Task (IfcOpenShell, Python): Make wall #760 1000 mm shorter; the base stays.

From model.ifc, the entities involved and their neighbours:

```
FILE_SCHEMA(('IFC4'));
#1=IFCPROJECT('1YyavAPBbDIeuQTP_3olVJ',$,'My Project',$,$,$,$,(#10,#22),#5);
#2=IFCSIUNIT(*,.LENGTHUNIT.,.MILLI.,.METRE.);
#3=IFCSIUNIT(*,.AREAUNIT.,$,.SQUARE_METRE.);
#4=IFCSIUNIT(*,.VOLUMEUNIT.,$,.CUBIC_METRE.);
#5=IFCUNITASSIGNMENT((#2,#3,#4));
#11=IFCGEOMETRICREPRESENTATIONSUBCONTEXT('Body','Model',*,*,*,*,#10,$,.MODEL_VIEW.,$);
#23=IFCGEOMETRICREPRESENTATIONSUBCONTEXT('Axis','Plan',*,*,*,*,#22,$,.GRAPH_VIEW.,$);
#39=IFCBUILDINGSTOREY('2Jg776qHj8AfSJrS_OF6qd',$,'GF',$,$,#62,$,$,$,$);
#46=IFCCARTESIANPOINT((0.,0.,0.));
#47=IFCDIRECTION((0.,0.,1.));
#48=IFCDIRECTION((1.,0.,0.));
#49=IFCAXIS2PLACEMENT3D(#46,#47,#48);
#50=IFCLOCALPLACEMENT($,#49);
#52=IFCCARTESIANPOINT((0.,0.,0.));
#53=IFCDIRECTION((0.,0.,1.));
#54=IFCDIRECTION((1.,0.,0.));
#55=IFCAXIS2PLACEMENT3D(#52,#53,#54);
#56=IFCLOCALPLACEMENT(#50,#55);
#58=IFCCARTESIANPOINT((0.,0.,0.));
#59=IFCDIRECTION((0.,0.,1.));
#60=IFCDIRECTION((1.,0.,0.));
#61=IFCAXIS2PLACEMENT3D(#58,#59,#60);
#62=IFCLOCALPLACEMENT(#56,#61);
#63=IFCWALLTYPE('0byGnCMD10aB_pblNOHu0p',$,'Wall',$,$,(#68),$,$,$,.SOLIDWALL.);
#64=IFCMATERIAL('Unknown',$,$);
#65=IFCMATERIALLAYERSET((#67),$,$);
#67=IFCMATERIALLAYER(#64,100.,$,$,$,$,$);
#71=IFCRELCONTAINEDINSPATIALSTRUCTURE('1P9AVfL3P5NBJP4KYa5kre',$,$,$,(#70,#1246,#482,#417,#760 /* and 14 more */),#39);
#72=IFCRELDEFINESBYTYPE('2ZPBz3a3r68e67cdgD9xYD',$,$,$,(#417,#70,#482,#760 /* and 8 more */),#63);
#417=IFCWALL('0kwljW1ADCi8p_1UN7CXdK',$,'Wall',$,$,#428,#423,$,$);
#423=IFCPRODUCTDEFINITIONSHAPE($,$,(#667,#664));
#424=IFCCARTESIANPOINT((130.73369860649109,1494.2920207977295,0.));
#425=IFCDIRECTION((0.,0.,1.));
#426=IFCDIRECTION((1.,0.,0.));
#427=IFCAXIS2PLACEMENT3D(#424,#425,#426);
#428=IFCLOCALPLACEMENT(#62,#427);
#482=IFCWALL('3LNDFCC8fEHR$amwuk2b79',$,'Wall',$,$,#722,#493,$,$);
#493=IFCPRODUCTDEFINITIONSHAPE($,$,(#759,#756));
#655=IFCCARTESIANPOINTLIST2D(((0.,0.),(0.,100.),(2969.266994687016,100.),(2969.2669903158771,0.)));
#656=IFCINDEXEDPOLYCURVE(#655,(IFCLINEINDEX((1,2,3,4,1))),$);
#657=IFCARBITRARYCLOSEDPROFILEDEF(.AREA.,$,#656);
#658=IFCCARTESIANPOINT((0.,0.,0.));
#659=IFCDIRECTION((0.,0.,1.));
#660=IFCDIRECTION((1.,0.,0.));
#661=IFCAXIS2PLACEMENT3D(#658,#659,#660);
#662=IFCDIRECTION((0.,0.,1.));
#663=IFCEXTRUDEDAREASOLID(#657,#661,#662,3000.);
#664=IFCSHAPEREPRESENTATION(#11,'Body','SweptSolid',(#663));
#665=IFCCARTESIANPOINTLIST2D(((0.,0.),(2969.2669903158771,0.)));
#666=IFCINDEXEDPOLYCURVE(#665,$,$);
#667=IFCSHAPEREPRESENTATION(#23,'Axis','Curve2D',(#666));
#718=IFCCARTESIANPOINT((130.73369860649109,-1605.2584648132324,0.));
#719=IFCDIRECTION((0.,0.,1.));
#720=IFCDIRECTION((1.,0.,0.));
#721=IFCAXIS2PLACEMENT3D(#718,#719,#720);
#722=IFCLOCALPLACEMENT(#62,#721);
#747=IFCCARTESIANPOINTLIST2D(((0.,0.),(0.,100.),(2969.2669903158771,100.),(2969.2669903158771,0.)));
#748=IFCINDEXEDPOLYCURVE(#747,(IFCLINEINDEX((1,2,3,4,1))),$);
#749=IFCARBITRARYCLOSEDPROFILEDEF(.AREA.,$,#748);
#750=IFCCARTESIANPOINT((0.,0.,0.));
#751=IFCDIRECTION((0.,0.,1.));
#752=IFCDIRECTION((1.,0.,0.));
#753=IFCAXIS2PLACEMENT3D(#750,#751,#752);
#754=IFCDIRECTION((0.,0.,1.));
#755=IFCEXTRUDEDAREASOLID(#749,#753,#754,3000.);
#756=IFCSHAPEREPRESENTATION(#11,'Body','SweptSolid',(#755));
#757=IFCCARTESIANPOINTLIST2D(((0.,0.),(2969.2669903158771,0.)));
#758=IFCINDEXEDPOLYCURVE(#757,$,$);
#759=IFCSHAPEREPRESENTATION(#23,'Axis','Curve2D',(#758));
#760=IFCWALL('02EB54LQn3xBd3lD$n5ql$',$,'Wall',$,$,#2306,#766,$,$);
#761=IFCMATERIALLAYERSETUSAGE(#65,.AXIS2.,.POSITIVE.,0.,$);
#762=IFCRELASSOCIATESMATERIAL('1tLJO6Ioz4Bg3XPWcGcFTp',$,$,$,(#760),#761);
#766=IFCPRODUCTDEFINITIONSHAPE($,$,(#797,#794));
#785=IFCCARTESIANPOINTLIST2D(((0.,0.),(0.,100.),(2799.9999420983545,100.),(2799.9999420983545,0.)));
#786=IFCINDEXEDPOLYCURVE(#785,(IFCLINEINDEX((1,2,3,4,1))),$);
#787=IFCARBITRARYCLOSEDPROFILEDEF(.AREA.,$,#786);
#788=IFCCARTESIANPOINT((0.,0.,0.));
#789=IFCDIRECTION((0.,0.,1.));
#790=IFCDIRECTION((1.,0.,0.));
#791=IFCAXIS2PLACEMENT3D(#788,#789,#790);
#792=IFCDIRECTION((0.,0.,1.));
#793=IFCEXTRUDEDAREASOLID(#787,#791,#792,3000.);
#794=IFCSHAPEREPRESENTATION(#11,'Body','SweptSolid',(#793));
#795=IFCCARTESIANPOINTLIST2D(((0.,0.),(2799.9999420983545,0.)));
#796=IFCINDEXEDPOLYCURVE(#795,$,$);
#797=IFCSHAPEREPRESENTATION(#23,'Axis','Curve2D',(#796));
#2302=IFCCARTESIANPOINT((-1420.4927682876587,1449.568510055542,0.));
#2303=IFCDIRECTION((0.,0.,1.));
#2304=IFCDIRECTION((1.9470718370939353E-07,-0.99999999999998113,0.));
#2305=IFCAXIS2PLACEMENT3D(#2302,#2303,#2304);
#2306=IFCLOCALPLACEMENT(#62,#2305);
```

```python
import ifcopenshell
import ifcopenshell.geom
import ifcopenshell.util.representation
import ifcopenshell.util.shape
import ifcopenshell.util.unit

model = ifcopenshell.open("model.ifc")
unit_scale = ifcopenshell.util.unit.calculate_unit_scale(model)
settings = ifcopenshell.geom.settings()


def volume(element):
    """Net volume in cubic metres, openings subtracted."""
    shape = ifcopenshell.geom.create_shape(settings, element)
    return ifcopenshell.util.shape.get_volume(shape.geometry)


wall = model.by_id(760)
before = volume(wall)

body = ifcopenshell.util.representation.get_representation(wall, "Model", "Body")
solid = body.Items[0]
old_height = solid.Depth
solid.Depth -= 1 / unit_scale
after = volume(wall)

print(f"height {old_height:g} -> {solid.Depth:g}, volume {before:.3f} -> {after:.3f} m3")

model.write("model_rev.ifc")
```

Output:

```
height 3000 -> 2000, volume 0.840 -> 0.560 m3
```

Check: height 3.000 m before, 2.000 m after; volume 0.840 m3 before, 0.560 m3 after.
